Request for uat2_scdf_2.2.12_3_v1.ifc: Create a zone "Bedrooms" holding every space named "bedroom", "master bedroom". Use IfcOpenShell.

First a look at what the model holds.

```python
import ifcopenshell

model = ifcopenshell.open("uat2_scdf_2.2.12_3_v1.ifc")
print(model.schema)
seen = {}
for space in model.by_type("IfcSpace"):
    seen[space.LongName] = seen.get(space.LongName, 0) + 1
for name, count in sorted(seen.items(), key=str):
    print(count, "x", name)
print("zones:", [z.Name for z in model.by_type("IfcZone")][:20])
```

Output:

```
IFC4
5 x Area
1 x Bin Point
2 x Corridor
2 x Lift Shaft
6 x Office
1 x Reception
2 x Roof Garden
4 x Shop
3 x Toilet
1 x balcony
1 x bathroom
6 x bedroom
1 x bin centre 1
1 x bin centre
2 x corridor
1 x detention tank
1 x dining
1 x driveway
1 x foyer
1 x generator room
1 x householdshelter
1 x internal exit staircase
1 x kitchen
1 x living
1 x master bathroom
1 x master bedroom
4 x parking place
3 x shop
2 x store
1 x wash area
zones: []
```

```python
import ifcopenshell
import ifcopenshell.api.group
import ifcopenshell.api.root

model = ifcopenshell.open("uat2_scdf_2.2.12_3_v1.ifc")

names = {"bedroom", "master bedroom"}
spaces = [s for s in model.by_type("IfcSpace") if s.LongName in names]

zone = ifcopenshell.api.root.create_entity(model, ifc_class="IfcZone", name="Bedrooms")
ifcopenshell.api.group.assign_group(model, products=spaces, group=zone)
print(len(spaces), "spaces in", zone.Name)

model.write("uat2_scdf_2.2.12_3_v1_edited.ifc")
```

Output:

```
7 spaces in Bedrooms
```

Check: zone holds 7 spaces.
